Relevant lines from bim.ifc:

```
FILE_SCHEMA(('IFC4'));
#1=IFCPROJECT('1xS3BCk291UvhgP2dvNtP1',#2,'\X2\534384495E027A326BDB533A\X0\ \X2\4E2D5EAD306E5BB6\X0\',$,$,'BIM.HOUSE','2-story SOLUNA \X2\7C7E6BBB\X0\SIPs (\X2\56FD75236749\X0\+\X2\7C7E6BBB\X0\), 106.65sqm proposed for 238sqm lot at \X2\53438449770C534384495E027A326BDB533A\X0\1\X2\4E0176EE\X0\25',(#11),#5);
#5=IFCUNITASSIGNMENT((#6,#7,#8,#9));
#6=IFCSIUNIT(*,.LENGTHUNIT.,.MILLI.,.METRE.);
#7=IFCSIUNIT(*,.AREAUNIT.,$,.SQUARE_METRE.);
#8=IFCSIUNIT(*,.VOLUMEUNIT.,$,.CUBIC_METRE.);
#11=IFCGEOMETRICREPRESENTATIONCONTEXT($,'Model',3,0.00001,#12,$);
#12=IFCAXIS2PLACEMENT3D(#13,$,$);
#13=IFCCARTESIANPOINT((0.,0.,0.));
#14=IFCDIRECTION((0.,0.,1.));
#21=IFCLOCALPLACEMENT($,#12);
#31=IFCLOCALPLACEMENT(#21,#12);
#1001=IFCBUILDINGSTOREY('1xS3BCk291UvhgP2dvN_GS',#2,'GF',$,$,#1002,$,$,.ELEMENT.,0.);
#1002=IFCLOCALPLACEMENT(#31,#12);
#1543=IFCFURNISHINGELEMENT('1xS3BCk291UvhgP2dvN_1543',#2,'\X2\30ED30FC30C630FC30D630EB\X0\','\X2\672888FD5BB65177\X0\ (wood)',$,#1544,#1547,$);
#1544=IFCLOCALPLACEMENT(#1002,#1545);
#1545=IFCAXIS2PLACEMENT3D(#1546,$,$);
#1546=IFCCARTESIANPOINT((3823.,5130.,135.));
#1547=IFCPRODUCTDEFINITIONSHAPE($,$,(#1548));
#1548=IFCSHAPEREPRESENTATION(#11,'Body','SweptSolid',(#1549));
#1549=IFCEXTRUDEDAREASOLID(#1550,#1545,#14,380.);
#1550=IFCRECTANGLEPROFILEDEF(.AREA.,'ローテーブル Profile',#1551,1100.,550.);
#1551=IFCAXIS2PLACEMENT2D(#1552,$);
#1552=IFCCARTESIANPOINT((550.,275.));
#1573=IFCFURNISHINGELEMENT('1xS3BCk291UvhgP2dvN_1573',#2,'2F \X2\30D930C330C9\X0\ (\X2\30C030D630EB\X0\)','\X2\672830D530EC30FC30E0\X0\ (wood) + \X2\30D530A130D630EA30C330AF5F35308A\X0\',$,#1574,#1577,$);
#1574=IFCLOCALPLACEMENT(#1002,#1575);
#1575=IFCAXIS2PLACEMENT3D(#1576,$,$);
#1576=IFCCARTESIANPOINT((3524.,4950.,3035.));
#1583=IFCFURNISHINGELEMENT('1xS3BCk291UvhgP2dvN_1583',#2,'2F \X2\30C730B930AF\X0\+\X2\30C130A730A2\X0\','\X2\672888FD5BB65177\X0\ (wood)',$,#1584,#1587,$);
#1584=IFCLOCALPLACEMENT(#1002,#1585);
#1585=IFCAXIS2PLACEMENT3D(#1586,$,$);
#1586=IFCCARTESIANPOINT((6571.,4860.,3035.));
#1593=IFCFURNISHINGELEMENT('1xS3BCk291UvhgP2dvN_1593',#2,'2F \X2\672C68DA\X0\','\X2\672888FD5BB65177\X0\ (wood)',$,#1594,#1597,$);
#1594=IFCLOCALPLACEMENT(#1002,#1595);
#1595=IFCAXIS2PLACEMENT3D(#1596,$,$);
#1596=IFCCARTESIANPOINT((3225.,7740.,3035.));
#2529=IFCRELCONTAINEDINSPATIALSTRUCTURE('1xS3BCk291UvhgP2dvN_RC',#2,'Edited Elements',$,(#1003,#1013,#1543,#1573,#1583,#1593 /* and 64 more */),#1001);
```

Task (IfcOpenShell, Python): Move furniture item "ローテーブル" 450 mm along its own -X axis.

```python
import ifcopenshell
import ifcopenshell.api.geometry
import ifcopenshell.util.placement
import ifcopenshell.util.unit

model = ifcopenshell.open("bim.ifc")
unit_scale = ifcopenshell.util.unit.calculate_unit_scale(model)

item = model.by_id(1543)
matrix = ifcopenshell.util.placement.get_local_placement(item.ObjectPlacement)
matrix[:3, 3] -= matrix[:3, 0] * 0.45 / unit_scale
ifcopenshell.api.geometry.edit_object_placement(model, product=item, matrix=matrix, is_si=False)

print(ifcopenshell.util.placement.get_local_placement(item.ObjectPlacement).round(3) + 0.0)

model.write("bim_updated.ifc")
```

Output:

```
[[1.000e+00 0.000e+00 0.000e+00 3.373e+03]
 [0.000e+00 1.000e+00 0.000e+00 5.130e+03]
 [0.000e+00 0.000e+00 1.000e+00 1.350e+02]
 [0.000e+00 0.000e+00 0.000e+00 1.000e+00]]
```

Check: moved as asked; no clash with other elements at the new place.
